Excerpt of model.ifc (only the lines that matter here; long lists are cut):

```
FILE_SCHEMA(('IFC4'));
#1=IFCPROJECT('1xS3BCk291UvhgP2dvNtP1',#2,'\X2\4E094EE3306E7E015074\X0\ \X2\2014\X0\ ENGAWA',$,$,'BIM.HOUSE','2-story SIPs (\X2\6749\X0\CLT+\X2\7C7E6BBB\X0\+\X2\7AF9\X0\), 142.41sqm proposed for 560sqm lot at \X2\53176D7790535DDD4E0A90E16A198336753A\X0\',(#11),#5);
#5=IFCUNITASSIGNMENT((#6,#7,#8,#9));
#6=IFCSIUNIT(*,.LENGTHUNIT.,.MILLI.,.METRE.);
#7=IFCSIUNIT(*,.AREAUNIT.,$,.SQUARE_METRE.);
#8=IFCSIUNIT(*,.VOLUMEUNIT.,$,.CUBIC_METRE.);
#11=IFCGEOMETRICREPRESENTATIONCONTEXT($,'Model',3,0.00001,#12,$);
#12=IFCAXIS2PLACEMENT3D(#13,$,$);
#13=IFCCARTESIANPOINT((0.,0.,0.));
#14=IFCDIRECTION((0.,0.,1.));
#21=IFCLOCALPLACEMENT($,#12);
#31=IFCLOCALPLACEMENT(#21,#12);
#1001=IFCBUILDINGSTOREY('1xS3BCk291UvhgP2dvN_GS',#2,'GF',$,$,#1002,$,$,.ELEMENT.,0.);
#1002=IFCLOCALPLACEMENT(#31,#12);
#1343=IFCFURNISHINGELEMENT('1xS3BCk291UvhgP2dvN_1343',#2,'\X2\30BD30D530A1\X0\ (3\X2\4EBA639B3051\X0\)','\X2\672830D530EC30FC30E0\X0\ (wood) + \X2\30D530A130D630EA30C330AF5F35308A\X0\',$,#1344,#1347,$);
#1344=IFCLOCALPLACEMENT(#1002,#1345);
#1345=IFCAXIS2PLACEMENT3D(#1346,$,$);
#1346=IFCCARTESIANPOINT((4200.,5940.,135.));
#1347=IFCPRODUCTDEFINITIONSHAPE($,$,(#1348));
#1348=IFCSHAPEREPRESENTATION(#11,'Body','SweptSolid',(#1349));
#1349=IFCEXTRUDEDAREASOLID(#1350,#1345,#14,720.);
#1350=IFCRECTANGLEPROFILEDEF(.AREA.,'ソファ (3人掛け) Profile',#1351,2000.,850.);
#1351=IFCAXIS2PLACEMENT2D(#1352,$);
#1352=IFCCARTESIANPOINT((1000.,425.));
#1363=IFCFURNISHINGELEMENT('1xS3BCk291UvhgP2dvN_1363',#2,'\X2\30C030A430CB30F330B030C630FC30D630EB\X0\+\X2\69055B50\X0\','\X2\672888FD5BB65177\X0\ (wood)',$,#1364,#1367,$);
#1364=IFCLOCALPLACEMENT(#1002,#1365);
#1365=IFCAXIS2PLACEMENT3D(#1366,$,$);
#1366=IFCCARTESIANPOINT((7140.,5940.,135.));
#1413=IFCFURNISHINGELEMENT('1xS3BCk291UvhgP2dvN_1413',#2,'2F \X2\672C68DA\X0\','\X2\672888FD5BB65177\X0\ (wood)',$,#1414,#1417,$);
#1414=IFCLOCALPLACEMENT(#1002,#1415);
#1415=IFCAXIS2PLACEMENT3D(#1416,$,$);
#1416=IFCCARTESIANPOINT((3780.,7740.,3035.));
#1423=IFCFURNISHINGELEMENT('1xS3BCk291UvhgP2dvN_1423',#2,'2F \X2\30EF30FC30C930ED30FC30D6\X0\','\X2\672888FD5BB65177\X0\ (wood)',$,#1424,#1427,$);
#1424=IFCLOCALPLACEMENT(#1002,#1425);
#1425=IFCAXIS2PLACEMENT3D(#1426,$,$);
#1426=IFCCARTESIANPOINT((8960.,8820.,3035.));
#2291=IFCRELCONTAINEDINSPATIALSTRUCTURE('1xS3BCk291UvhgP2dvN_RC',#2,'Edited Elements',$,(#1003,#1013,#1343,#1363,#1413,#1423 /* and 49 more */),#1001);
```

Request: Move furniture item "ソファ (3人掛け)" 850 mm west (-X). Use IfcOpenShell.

```python
import ifcopenshell
import ifcopenshell.api.geometry
import ifcopenshell.util.placement
import ifcopenshell.util.unit

model = ifcopenshell.open("model.ifc")
unit_scale = ifcopenshell.util.unit.calculate_unit_scale(model)

item = model.by_id(1343)
matrix = ifcopenshell.util.placement.get_local_placement(item.ObjectPlacement)
matrix[0, 3] -= 0.85 / unit_scale
ifcopenshell.api.geometry.edit_object_placement(model, product=item, matrix=matrix, is_si=False)

print(ifcopenshell.util.placement.get_local_placement(item.ObjectPlacement).round(3) + 0.0)

model.write("model_v2.ifc")
```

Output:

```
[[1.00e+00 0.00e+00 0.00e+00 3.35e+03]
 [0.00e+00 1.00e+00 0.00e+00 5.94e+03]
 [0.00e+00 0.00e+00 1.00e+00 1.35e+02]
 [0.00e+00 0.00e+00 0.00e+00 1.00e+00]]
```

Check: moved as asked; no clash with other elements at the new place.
